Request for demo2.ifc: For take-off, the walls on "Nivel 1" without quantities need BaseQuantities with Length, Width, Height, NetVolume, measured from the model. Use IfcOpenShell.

First a look at what the model holds.

```python
import ifcopenshell
import ifcopenshell.util.element
import ifcopenshell.util.unit

model = ifcopenshell.open("demo2.ifc")
print(model.schema)
for unit_type in ("LENGTHUNIT", "AREAUNIT", "VOLUMEUNIT"):
    print(unit_type, ifcopenshell.util.unit.calculate_unit_scale(model, unit_type))
storey = next(s for s in model.by_type("IfcBuildingStorey") if s.Name == "Nivel 1")
walls = [e for e in ifcopenshell.util.element.get_decomposition(storey) if e.is_a("IfcWall")]
for e in sorted(walls, key=lambda e: e.id()):
    print(e.id(), e.is_a(), e.Name, list(ifcopenshell.util.element.get_psets(e, qtos_only=True)), sep=" | ")
```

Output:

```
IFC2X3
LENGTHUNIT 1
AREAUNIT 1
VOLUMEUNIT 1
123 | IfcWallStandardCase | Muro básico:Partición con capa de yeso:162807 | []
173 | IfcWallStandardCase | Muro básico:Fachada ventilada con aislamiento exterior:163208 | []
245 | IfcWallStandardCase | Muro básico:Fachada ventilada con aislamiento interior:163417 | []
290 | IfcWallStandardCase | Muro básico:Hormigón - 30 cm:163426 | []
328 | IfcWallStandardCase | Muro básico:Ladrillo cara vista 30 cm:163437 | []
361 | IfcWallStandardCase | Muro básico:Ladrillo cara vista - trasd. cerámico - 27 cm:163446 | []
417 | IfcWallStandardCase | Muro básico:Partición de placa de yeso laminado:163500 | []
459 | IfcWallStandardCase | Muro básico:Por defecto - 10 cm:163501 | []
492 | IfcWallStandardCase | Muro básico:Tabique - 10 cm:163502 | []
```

```python
import ifcopenshell
import ifcopenshell.api.pset
import ifcopenshell.geom
import ifcopenshell.util.element
import ifcopenshell.util.shape
import ifcopenshell.util.unit

model = ifcopenshell.open("demo2.ifc")
unit_scale = ifcopenshell.util.unit.calculate_unit_scale(model)
volume_scale = ifcopenshell.util.unit.calculate_unit_scale(model, "VOLUMEUNIT")
settings = ifcopenshell.geom.settings()

storey = next(s for s in model.by_type("IfcBuildingStorey") if s.Name == "Nivel 1")
walls = [e for e in ifcopenshell.util.element.get_decomposition(storey) if e.is_a("IfcWall")]

for e in sorted(walls, key=lambda e: e.id()):
    if ifcopenshell.util.element.get_psets(e, qtos_only=True, should_inherit=False):
        continue
    # Geometry comes back in metres, in the element's own axes.
    shape = ifcopenshell.geom.create_shape(settings, e)
    values = {
        "Length": ifcopenshell.util.shape.get_x(shape.geometry) / unit_scale,
        "Width": ifcopenshell.util.shape.get_y(shape.geometry) / unit_scale,
        "Height": ifcopenshell.util.shape.get_z(shape.geometry) / unit_scale,
        "NetVolume": ifcopenshell.util.shape.get_volume(shape.geometry) / volume_scale,
    }
    qto = ifcopenshell.api.pset.add_qto(model, product=e, name="BaseQuantities")
    ifcopenshell.api.pset.edit_qto(model, qto=qto, properties=values)
    print(e.id(), {k: round(v, 3) for k, v in values.items()})

model.write("demo2_rev.ifc")
```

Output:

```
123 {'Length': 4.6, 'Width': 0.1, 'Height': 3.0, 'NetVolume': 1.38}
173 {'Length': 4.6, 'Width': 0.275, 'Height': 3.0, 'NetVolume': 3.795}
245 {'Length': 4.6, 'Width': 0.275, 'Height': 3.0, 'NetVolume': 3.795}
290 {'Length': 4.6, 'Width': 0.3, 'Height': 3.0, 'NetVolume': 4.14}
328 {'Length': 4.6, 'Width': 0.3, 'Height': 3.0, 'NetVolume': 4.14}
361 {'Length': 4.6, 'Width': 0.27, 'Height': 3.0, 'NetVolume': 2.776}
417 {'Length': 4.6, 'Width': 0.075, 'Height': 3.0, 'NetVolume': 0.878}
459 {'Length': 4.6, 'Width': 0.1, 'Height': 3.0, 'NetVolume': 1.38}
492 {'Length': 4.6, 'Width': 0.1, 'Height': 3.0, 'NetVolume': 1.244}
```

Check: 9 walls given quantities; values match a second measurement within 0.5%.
